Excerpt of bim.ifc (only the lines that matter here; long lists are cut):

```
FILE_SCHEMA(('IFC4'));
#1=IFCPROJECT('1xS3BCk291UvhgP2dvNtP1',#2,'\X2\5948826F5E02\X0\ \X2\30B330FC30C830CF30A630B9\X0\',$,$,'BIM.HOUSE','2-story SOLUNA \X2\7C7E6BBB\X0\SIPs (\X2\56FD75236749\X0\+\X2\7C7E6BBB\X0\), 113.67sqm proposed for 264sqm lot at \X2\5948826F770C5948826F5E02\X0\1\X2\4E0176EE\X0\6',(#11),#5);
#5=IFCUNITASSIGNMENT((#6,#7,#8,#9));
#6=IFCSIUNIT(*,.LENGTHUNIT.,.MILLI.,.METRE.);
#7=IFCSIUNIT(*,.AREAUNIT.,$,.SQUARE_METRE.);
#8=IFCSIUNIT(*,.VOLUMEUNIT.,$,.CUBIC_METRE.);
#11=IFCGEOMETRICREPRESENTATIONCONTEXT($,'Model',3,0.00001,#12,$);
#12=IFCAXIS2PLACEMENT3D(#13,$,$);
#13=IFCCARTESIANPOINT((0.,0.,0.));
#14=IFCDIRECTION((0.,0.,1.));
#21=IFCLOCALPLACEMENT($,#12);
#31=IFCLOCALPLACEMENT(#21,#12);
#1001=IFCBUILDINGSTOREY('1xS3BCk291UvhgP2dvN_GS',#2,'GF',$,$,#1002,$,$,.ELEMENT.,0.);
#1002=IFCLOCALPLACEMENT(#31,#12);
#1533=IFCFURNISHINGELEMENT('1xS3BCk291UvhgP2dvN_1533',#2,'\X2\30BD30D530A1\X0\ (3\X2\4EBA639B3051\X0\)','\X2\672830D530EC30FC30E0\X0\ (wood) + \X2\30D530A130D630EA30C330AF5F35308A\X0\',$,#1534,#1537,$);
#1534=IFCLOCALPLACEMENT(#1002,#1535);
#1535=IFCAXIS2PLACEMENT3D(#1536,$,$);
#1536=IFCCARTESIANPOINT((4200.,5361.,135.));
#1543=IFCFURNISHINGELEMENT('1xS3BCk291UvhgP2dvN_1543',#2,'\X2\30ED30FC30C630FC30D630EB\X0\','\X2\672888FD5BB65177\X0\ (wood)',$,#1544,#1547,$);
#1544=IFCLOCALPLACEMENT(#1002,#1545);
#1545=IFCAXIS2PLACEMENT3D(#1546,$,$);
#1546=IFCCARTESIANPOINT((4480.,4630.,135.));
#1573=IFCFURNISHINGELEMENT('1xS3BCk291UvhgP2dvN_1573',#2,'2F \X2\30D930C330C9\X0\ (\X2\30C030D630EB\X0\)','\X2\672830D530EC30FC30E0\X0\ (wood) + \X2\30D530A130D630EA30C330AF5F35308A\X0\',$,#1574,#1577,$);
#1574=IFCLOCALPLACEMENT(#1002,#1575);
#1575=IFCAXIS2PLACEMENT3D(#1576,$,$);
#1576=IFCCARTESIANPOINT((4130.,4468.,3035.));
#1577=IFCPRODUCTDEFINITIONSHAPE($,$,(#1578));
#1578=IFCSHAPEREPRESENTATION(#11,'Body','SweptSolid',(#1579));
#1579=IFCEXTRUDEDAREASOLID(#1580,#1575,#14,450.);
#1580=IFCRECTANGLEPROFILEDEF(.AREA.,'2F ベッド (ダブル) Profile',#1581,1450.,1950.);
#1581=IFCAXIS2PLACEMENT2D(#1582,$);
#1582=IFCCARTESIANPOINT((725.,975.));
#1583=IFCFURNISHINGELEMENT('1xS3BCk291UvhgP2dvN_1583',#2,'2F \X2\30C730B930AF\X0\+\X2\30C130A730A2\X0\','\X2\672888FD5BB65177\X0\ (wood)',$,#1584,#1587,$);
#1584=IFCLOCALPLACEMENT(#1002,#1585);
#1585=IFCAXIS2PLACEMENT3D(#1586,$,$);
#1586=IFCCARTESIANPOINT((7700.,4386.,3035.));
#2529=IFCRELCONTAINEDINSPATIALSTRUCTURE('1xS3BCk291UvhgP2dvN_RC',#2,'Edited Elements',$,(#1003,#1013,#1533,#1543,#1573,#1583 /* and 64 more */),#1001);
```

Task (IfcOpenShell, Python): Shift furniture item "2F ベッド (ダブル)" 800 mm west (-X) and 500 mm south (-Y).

```python
import ifcopenshell
import ifcopenshell.api.geometry
import ifcopenshell.util.placement
import ifcopenshell.util.unit

model = ifcopenshell.open("bim.ifc")
unit_scale = ifcopenshell.util.unit.calculate_unit_scale(model)

item = model.by_guid("1xS3BCk291UvhgP2dvN_1573")
matrix = ifcopenshell.util.placement.get_local_placement(item.ObjectPlacement)
matrix[0, 3] -= 0.8 / unit_scale
matrix[1, 3] -= 0.5 / unit_scale
ifcopenshell.api.geometry.edit_object_placement(model, product=item, matrix=matrix, is_si=False)

print(ifcopenshell.util.placement.get_local_placement(item.ObjectPlacement).round(3) + 0.0)

model.write("bim_rev.ifc")
```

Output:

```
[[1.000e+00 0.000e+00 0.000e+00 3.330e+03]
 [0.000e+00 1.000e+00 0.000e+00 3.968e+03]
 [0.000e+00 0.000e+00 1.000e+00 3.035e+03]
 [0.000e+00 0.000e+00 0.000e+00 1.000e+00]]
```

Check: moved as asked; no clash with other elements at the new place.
